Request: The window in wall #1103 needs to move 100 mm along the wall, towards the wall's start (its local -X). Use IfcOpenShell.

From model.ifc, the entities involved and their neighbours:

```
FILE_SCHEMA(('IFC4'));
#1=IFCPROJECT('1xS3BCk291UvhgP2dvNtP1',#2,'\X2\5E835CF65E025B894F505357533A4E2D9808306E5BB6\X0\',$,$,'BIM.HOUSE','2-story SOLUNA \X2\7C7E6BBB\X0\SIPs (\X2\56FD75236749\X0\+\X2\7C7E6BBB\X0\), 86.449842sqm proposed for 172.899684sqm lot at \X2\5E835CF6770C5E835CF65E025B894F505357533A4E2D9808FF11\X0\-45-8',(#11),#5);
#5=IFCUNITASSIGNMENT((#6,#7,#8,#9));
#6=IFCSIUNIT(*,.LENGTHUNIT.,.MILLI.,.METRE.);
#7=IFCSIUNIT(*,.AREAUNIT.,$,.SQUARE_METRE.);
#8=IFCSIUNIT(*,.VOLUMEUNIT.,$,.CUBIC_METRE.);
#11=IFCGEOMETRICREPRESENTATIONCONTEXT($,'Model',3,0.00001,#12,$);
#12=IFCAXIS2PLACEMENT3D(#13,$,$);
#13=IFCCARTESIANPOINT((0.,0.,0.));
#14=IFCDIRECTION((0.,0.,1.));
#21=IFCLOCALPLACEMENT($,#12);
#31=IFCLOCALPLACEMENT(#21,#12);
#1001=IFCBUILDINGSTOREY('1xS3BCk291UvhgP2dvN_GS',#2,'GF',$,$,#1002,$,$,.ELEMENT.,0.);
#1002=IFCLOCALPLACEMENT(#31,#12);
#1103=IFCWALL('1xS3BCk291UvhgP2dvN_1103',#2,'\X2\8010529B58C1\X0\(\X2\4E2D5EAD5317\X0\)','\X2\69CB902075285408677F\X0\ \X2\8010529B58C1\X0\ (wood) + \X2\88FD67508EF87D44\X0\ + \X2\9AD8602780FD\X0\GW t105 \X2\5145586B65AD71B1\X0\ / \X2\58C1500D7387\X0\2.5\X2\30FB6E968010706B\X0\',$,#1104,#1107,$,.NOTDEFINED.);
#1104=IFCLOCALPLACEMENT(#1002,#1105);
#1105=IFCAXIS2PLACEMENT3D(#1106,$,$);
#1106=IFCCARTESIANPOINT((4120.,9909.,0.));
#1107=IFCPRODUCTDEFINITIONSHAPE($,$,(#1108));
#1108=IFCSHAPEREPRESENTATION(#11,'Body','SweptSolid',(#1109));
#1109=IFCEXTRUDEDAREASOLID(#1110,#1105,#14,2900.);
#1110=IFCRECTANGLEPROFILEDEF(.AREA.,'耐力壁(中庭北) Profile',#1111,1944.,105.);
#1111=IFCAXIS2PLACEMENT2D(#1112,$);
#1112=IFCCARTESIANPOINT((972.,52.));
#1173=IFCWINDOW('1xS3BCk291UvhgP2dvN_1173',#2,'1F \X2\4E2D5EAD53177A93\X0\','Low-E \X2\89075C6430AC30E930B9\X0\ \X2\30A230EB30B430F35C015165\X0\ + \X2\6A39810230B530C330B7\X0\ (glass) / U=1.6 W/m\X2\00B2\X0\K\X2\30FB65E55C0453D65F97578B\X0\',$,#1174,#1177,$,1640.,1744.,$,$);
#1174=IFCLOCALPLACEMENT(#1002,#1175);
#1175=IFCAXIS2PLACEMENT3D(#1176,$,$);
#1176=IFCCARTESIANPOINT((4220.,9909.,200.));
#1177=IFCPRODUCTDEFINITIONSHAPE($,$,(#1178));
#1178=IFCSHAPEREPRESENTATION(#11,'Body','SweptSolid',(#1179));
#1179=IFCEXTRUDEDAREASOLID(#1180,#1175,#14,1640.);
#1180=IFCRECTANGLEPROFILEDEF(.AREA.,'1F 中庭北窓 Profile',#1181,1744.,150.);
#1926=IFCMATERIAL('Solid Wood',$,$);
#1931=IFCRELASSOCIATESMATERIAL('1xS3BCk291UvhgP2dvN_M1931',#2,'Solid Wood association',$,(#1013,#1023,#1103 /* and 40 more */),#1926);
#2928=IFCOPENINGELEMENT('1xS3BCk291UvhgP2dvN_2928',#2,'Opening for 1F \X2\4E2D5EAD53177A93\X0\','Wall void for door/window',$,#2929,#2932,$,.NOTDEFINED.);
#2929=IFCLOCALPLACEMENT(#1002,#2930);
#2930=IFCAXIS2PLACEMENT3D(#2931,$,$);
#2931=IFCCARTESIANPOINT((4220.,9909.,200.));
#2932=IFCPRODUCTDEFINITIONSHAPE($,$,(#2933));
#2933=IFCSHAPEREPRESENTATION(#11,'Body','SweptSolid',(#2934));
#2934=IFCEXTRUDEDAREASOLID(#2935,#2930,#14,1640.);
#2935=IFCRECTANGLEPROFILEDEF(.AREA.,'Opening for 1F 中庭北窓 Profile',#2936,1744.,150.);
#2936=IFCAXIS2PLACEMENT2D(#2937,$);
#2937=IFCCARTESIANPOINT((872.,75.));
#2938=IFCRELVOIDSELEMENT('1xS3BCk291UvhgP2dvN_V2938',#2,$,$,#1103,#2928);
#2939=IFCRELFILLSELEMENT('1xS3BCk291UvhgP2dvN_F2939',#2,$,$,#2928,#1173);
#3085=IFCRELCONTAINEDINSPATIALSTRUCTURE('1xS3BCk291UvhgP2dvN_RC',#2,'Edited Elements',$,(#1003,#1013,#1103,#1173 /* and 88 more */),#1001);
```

```python
import ifcopenshell
import ifcopenshell.api.geometry
import ifcopenshell.util.placement

model = ifcopenshell.open("model.ifc")

window = model.by_guid("1xS3BCk291UvhgP2dvN_1173")
opening = window.FillsVoids[0].RelatingOpeningElement
wall = opening.VoidsElements[0].RelatingBuildingElement

wall_matrix = ifcopenshell.util.placement.get_local_placement(wall.ObjectPlacement)
shift = wall_matrix[:3, 0] * -100.0
before = ifcopenshell.util.placement.get_local_placement(window.ObjectPlacement)[:3, 3].copy()

# The window is not placed relative to its opening, so move both.
for product in (opening, window):
    matrix = ifcopenshell.util.placement.get_local_placement(product.ObjectPlacement)
    matrix[:3, 3] += shift
    ifcopenshell.api.geometry.edit_object_placement(model, product=product, matrix=matrix, is_si=False)

after = ifcopenshell.util.placement.get_local_placement(window.ObjectPlacement)[:3, 3]
print("window moved by", (after - before).round(3) + 0.0)

model.write("model-out.ifc")
```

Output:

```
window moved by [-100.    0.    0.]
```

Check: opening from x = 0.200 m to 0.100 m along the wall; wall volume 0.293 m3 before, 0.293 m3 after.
